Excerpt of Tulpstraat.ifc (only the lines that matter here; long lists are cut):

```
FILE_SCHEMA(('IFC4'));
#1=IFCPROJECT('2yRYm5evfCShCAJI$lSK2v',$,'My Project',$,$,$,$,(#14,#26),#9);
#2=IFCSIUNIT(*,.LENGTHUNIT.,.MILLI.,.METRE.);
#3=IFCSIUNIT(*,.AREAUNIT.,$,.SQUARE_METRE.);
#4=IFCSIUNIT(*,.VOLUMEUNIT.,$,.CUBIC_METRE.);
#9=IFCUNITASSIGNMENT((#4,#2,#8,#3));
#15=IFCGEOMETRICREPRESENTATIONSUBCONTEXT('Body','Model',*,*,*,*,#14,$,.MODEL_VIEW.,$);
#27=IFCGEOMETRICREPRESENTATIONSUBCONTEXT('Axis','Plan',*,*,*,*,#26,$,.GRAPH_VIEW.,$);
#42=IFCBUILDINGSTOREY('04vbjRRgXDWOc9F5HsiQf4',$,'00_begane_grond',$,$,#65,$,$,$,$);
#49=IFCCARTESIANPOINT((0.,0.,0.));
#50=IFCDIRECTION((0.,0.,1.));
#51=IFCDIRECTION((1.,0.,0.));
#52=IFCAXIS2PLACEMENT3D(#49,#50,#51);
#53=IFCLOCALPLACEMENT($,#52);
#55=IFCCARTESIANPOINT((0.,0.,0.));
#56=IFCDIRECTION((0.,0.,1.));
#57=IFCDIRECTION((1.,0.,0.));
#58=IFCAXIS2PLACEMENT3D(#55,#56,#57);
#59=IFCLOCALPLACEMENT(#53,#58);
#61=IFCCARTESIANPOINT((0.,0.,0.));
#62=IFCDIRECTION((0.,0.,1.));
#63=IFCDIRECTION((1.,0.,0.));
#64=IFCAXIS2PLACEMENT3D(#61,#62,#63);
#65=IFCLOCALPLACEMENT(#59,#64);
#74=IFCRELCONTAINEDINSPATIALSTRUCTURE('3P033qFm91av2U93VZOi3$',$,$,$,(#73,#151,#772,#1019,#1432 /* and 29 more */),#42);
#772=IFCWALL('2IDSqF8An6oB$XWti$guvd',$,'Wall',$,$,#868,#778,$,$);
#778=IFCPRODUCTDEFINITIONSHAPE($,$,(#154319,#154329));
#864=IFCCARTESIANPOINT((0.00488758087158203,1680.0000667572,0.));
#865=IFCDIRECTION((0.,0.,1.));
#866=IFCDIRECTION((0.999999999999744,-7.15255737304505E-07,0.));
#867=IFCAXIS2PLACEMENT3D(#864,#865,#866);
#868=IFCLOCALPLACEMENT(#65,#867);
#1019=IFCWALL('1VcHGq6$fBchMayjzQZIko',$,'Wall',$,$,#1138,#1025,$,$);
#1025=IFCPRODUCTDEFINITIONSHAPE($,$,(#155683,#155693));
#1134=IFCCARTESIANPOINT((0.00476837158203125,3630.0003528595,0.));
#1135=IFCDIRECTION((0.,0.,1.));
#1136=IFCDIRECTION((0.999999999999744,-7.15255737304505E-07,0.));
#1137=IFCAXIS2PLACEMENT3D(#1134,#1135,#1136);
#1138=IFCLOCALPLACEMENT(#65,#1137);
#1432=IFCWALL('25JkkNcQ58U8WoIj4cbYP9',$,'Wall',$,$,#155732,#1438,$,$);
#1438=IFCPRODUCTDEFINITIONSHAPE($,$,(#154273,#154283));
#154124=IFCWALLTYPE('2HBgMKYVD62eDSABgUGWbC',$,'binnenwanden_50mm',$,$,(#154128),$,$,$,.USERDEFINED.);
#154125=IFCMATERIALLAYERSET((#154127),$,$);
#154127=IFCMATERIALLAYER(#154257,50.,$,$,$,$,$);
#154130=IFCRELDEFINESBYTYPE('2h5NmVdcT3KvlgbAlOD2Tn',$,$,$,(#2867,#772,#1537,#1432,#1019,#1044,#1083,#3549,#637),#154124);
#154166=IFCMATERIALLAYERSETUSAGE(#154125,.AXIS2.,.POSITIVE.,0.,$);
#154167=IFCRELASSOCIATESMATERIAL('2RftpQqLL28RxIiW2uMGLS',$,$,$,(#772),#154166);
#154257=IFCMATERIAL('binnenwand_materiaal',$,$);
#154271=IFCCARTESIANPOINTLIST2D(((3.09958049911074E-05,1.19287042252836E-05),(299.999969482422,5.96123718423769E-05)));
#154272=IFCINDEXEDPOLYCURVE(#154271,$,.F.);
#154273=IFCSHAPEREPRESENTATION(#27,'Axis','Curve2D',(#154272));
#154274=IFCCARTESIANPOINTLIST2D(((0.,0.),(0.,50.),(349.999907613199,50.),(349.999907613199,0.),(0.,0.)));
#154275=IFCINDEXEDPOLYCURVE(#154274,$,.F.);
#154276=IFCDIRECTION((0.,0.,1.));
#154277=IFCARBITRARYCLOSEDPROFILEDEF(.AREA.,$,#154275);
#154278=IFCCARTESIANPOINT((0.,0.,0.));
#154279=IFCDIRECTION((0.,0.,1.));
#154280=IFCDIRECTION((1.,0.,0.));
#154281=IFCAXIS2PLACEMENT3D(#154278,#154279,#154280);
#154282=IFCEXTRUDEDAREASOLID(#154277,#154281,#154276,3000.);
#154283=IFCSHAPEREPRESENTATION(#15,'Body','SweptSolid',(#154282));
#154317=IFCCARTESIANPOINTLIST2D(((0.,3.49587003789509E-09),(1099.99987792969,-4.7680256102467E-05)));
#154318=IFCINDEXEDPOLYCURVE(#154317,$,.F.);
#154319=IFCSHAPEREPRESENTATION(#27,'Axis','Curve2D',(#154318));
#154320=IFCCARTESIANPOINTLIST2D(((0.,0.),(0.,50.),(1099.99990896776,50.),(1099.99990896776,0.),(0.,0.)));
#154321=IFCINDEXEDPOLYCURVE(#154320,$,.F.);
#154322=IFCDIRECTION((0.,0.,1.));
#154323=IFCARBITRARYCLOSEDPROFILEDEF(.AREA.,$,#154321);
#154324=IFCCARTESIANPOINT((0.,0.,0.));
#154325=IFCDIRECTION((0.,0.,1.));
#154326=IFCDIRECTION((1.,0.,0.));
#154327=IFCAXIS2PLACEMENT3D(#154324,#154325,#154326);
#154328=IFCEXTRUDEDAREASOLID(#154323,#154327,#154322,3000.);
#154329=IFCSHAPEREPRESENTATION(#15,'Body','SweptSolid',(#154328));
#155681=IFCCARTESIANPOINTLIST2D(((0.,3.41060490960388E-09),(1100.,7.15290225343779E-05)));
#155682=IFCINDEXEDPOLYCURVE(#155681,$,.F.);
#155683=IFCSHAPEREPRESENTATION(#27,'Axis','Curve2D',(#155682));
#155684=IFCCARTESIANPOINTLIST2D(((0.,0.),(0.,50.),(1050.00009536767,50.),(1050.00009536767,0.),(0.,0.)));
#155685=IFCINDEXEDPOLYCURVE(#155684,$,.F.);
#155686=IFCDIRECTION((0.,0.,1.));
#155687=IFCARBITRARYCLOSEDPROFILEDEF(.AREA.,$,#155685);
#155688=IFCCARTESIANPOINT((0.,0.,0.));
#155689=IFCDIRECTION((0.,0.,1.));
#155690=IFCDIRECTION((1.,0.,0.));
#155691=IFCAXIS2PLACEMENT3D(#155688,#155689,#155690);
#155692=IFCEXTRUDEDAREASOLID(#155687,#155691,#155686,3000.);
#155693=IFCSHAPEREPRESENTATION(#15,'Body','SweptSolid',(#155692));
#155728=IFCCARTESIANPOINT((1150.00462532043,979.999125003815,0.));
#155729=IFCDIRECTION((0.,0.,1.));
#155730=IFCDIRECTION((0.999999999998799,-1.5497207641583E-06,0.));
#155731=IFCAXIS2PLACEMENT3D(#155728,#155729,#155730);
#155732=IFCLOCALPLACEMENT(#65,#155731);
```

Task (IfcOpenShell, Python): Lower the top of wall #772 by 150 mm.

```python
import ifcopenshell
import ifcopenshell.geom
import ifcopenshell.util.representation
import ifcopenshell.util.shape
import ifcopenshell.util.unit

model = ifcopenshell.open("Tulpstraat.ifc")
unit_scale = ifcopenshell.util.unit.calculate_unit_scale(model)
settings = ifcopenshell.geom.settings()


def volume(element):
    """Net volume in cubic metres, openings subtracted."""
    shape = ifcopenshell.geom.create_shape(settings, element)
    return ifcopenshell.util.shape.get_volume(shape.geometry)


wall = model.by_guid("2IDSqF8An6oB$XWti$guvd")
before = volume(wall)

body = ifcopenshell.util.representation.get_representation(wall, "Model", "Body")
solid = body.Items[0]
old_height = solid.Depth
solid.Depth -= 0.15 / unit_scale
after = volume(wall)

print(f"height {old_height:g} -> {solid.Depth:g}, volume {before:.3f} -> {after:.3f} m3")

model.write("Tulpstraat-out.ifc")
```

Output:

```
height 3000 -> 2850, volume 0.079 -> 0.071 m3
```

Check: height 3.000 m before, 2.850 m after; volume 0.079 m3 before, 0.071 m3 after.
